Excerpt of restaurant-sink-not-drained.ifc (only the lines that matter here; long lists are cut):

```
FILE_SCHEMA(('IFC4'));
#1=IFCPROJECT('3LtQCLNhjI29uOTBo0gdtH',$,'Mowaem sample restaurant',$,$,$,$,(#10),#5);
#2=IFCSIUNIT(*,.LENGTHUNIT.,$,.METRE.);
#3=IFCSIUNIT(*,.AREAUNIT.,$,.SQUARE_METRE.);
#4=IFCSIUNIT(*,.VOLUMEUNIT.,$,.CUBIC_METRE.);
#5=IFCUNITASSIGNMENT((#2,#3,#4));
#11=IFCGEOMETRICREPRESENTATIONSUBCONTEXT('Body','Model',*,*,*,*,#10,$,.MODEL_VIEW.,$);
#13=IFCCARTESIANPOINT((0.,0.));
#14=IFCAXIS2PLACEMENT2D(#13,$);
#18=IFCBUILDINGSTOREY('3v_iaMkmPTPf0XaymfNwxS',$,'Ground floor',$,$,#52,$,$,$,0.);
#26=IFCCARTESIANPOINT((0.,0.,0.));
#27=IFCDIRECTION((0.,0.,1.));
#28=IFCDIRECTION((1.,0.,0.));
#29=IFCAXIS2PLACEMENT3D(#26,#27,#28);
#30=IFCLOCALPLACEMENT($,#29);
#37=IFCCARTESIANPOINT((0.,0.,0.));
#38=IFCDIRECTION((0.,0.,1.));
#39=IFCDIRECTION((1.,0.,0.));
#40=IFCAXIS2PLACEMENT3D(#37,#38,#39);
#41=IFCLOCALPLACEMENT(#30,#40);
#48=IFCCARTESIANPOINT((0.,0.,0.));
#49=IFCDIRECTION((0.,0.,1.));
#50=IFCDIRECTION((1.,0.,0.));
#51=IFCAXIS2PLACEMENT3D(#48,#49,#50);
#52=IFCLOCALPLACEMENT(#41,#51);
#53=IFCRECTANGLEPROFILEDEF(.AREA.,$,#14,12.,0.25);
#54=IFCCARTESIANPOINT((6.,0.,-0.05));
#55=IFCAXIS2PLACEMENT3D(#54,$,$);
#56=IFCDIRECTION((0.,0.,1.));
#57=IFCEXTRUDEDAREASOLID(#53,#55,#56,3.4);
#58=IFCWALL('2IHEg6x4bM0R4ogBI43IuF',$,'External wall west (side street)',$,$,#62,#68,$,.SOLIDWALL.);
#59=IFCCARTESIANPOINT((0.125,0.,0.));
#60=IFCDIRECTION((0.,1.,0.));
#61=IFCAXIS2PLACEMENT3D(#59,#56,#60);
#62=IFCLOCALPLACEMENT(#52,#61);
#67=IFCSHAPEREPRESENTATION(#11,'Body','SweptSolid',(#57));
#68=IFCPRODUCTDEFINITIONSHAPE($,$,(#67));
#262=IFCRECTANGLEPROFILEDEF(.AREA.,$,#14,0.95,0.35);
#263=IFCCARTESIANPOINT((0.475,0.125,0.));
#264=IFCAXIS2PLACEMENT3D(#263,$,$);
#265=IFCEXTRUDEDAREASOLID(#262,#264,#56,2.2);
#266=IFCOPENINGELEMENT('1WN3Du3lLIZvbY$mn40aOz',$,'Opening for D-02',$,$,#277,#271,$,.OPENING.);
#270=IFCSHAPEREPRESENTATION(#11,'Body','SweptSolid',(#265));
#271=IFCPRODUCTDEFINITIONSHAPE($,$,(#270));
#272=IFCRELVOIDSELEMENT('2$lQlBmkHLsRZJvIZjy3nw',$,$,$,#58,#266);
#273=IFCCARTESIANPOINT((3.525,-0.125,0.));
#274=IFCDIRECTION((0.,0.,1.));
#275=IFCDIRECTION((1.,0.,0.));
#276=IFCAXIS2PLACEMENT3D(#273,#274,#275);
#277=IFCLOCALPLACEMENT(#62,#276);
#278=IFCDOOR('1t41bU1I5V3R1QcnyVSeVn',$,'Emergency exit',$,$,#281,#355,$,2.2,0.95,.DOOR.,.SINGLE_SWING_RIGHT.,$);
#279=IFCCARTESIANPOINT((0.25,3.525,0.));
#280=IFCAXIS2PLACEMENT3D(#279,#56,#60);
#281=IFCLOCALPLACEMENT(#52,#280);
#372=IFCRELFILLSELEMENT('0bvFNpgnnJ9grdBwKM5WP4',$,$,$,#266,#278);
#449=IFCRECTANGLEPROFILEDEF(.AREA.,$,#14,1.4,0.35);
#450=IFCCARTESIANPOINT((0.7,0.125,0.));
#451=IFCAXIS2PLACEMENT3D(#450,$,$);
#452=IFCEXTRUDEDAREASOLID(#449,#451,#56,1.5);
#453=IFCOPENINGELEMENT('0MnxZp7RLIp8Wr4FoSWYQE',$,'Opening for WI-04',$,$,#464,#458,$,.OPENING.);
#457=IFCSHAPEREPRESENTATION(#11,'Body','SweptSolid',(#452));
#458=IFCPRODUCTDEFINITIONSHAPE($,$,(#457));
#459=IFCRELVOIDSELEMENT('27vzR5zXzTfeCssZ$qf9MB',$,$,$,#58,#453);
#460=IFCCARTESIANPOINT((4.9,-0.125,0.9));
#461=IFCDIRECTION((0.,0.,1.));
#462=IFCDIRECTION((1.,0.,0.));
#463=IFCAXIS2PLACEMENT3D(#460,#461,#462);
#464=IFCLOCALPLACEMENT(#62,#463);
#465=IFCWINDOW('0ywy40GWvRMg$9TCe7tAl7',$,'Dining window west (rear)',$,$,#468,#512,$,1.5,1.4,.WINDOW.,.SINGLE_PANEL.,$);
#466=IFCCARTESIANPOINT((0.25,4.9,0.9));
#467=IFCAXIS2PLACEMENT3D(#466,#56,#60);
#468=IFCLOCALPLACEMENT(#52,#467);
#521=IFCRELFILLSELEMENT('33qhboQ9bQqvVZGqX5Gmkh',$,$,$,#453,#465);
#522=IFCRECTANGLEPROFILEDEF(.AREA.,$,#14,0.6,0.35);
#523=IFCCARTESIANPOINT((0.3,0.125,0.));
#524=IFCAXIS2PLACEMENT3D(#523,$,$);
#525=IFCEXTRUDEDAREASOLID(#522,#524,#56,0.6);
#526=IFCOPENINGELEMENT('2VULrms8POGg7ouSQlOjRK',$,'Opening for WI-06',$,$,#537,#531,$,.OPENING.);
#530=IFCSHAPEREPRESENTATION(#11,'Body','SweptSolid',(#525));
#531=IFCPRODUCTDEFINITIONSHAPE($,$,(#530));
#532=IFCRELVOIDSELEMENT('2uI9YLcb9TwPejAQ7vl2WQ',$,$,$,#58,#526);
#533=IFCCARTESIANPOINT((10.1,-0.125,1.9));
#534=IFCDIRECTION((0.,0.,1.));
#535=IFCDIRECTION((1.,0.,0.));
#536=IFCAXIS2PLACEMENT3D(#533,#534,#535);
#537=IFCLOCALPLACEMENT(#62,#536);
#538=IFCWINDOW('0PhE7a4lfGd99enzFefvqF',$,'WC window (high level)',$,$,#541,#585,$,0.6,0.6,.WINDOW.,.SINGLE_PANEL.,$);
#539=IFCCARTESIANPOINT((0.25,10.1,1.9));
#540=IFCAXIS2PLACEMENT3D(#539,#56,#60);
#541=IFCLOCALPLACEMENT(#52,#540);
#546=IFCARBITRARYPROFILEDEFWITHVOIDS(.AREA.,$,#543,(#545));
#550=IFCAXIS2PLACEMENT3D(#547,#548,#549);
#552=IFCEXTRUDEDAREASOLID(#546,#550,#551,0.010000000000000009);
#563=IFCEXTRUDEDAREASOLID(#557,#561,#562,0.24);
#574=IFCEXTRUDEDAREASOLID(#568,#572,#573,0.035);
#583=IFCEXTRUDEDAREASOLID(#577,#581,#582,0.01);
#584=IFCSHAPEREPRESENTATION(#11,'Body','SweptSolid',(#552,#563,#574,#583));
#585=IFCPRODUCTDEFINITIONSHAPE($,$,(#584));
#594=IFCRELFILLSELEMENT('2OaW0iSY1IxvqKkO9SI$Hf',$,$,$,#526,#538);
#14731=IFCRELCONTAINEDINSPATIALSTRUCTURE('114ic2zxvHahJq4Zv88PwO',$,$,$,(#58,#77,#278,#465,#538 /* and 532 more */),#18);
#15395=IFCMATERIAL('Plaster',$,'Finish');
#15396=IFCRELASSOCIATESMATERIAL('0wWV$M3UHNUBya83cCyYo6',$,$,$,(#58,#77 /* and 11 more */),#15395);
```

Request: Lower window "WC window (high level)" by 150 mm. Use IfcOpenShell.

```python
import numpy as np
import ifcopenshell
import ifcopenshell.api.geometry
import ifcopenshell.util.placement
import ifcopenshell.util.unit

model = ifcopenshell.open("restaurant-sink-not-drained.ifc")
unit_scale = ifcopenshell.util.unit.calculate_unit_scale(model)

window = model.by_id(538)
opening = window.FillsVoids[0].RelatingOpeningElement
dz = -0.15

shift = np.array([0.0, 0.0, dz])
# The window is not placed relative to its opening, so move both.
for product in (opening, window):
    matrix = ifcopenshell.util.placement.get_local_placement(product.ObjectPlacement)
    matrix[:3, 3] += shift
    ifcopenshell.api.geometry.edit_object_placement(model, product=product, matrix=matrix, is_si=False)

print(f"moved by {dz * unit_scale:+.3f} m")

model.write("restaurant-sink-not-drained-out.ifc")
```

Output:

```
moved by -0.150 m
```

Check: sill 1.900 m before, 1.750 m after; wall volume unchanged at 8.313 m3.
